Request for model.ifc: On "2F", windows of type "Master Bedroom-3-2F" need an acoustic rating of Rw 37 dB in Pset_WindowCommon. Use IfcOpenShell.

First a look at what the model holds.

```python
import ifcopenshell
import ifcopenshell.util.element

model = ifcopenshell.open("model.ifc")
print(model.schema)
storey = next(s for s in model.by_type("IfcBuildingStorey") if s.Name == "2F")
windows = [e for e in ifcopenshell.util.element.get_decomposition(storey) if e.is_a("IfcWindow")]
seen = {}
for e in windows:
    element_type = ifcopenshell.util.element.get_type(e)
    key = (element_type.Name if element_type != e and element_type else None, ifcopenshell.util.element.get_pset(e, "Pset_WindowCommon", "AcousticRating"))
    seen[key] = seen.get(key, 0) + 1
for (name, value), count in sorted(seen.items(), key=str):
    print(count, "x", name, "|", value)
```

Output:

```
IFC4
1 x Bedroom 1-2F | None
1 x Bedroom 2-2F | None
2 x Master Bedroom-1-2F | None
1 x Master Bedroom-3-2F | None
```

```python
import ifcopenshell
import ifcopenshell.api.pset
import ifcopenshell.util.element

model = ifcopenshell.open("model.ifc")

storey = next(s for s in model.by_type("IfcBuildingStorey") if s.Name == "2F")
windows = [e for e in ifcopenshell.util.element.get_decomposition(storey) if e.is_a("IfcWindow")]

count = 0
for e in windows:
    element_type = ifcopenshell.util.element.get_type(e)
    if element_type in (None, e) or element_type.Name != "Master Bedroom-3-2F":
        continue
    # add_pset returns the element's existing set when there is one.
    pset = ifcopenshell.api.pset.add_pset(model, product=e, name="Pset_WindowCommon")
    ifcopenshell.api.pset.edit_pset(model, pset=pset, properties={"AcousticRating": "Rw 37 dB"})
    count += 1

print(count, "windows updated")

model.write("model-out.ifc")
```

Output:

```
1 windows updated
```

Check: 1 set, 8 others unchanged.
